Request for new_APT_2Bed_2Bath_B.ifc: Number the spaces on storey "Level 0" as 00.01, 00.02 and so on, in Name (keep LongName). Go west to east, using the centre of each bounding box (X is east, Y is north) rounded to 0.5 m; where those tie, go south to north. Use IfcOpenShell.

First a look at what the model holds.

```python
import ifcopenshell
import ifcopenshell.util.element
import ifcopenshell.util.placement

model = ifcopenshell.open("new_APT_2Bed_2Bath_B.ifc")
print(model.schema)
storey = next(s for s in model.by_type("IfcBuildingStorey") if s.Name == "Level 0")
spaces = [e for e in ifcopenshell.util.element.get_decomposition(storey) if e.is_a("IfcSpace")]
for e in sorted(spaces, key=lambda e: e.id()):
    origin = ifcopenshell.util.placement.get_local_placement(e.ObjectPlacement)[:3, 3]
    print(e.id(), e.Name, e.LongName, origin.round(2) + 0.0, sep=" | ")
```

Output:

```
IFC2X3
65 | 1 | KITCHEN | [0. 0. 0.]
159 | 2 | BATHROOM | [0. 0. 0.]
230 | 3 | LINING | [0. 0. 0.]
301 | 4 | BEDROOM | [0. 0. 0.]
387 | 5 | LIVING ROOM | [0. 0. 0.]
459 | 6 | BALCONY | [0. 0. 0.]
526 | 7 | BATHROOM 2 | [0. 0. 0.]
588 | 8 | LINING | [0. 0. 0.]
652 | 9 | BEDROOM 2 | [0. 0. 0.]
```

```python
import ifcopenshell
import ifcopenshell.geom
import ifcopenshell.util.element
import ifcopenshell.util.shape

model = ifcopenshell.open("new_APT_2Bed_2Bath_B.ifc")
settings = ifcopenshell.geom.settings()
settings.set("use-world-coords", True)


def centre(element):
    shape = ifcopenshell.geom.create_shape(settings, element)
    return ifcopenshell.util.shape.get_bbox_centroid(shape.geometry)


storey = next(s for s in model.by_type("IfcBuildingStorey") if s.Name == "Level 0")
spaces = [e for e in ifcopenshell.util.element.get_decomposition(storey) if e.is_a("IfcSpace")]

# Insertion points can sit at a corner or the storey origin, so sort by the geometry (in metres).
centres = {e: centre(e) for e in spaces}
spaces.sort(key=lambda e: (round(centres[e][0] / 0.5), centres[e][1]))

for i, e in enumerate(spaces, start=1):
    number = f"00.{i:02d}"
    e.Name = number
    print(e.id(), number)

model.write("new_APT_2Bed_2Bath_B_rev.ifc")
```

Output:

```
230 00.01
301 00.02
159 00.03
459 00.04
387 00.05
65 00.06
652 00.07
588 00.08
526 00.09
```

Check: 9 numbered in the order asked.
